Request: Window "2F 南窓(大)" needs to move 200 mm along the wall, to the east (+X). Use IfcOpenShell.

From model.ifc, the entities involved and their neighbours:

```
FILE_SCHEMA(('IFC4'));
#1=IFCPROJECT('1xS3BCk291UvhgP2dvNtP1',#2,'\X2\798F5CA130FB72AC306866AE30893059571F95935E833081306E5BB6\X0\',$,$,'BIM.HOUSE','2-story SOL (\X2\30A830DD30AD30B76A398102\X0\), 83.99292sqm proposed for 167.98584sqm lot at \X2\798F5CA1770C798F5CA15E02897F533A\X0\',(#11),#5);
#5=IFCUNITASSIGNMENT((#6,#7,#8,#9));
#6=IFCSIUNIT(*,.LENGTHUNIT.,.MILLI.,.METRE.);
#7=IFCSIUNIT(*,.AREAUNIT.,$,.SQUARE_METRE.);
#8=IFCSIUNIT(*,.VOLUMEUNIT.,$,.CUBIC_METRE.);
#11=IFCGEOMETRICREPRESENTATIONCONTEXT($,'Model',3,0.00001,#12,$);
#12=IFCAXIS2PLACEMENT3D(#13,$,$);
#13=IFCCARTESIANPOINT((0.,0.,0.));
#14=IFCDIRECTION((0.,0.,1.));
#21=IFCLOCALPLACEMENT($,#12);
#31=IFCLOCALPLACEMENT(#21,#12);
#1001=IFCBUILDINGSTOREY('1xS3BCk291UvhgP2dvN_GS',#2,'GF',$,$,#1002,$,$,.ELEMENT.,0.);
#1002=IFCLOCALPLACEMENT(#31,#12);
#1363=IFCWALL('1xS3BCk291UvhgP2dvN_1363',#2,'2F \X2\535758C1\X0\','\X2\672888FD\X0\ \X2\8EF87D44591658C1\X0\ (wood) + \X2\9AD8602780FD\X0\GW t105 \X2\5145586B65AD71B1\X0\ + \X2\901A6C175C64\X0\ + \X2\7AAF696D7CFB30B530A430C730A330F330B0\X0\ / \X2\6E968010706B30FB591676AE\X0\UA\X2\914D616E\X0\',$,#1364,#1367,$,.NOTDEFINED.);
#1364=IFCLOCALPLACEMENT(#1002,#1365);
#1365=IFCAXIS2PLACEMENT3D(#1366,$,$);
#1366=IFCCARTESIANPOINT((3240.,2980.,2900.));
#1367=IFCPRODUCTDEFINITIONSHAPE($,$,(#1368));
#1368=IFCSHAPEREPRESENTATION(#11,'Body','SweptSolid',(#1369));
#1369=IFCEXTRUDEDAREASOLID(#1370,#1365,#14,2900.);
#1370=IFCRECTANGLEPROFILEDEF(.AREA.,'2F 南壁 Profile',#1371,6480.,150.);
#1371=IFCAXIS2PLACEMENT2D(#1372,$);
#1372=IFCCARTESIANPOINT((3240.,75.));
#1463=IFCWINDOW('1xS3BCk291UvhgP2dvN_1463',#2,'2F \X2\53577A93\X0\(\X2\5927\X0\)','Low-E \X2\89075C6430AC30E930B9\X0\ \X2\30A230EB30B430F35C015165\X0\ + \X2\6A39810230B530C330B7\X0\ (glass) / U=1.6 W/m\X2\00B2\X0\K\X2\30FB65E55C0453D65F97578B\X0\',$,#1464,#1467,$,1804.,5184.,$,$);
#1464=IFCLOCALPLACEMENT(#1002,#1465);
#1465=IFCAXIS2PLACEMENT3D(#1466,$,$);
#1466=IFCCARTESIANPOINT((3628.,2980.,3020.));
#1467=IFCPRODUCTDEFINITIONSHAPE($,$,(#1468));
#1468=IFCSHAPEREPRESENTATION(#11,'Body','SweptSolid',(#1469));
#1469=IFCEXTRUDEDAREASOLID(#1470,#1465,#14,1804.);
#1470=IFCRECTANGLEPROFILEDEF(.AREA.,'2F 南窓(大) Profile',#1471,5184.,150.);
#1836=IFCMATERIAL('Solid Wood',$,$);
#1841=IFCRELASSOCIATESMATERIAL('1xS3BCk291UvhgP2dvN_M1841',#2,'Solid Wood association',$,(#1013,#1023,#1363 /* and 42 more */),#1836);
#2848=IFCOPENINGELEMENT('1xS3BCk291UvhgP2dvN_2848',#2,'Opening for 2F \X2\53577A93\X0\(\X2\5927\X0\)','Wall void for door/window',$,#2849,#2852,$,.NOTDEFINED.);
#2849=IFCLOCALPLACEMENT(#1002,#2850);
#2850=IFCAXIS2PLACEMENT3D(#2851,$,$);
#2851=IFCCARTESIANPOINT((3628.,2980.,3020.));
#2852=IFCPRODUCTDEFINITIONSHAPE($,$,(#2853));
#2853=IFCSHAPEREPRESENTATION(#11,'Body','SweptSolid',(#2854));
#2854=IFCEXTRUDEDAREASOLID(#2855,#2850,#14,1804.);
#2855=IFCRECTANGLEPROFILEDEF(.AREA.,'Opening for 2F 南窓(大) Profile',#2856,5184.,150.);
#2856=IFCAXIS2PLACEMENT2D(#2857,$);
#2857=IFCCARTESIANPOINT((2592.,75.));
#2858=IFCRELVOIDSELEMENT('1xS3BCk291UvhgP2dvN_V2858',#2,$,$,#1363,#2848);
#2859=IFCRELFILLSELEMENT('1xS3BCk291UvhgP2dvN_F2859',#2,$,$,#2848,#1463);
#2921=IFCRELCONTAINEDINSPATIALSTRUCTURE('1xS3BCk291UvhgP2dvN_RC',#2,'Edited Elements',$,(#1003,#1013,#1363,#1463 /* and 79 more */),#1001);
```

```python
import ifcopenshell
import ifcopenshell.api.geometry
import ifcopenshell.util.placement
import ifcopenshell.util.unit

model = ifcopenshell.open("model.ifc")
unit_scale = ifcopenshell.util.unit.calculate_unit_scale(model)

window = model.by_guid("1xS3BCk291UvhgP2dvN_1463")
opening = window.FillsVoids[0].RelatingOpeningElement
wall = opening.VoidsElements[0].RelatingBuildingElement

wall_matrix = ifcopenshell.util.placement.get_local_placement(wall.ObjectPlacement)
shift = wall_matrix[:3, 0] * 0.2 / unit_scale
before = ifcopenshell.util.placement.get_local_placement(window.ObjectPlacement)[:3, 3].copy()

# The window is not placed relative to its opening, so move both.
for product in (opening, window):
    matrix = ifcopenshell.util.placement.get_local_placement(product.ObjectPlacement)
    matrix[:3, 3] += shift
    ifcopenshell.api.geometry.edit_object_placement(model, product=product, matrix=matrix, is_si=False)

after = ifcopenshell.util.placement.get_local_placement(window.ObjectPlacement)[:3, 3]
print("window moved by", (after - before).round(3) + 0.0)

model.write("model_v2.ifc")
```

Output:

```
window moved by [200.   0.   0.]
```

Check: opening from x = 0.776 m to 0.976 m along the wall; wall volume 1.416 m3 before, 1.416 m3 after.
